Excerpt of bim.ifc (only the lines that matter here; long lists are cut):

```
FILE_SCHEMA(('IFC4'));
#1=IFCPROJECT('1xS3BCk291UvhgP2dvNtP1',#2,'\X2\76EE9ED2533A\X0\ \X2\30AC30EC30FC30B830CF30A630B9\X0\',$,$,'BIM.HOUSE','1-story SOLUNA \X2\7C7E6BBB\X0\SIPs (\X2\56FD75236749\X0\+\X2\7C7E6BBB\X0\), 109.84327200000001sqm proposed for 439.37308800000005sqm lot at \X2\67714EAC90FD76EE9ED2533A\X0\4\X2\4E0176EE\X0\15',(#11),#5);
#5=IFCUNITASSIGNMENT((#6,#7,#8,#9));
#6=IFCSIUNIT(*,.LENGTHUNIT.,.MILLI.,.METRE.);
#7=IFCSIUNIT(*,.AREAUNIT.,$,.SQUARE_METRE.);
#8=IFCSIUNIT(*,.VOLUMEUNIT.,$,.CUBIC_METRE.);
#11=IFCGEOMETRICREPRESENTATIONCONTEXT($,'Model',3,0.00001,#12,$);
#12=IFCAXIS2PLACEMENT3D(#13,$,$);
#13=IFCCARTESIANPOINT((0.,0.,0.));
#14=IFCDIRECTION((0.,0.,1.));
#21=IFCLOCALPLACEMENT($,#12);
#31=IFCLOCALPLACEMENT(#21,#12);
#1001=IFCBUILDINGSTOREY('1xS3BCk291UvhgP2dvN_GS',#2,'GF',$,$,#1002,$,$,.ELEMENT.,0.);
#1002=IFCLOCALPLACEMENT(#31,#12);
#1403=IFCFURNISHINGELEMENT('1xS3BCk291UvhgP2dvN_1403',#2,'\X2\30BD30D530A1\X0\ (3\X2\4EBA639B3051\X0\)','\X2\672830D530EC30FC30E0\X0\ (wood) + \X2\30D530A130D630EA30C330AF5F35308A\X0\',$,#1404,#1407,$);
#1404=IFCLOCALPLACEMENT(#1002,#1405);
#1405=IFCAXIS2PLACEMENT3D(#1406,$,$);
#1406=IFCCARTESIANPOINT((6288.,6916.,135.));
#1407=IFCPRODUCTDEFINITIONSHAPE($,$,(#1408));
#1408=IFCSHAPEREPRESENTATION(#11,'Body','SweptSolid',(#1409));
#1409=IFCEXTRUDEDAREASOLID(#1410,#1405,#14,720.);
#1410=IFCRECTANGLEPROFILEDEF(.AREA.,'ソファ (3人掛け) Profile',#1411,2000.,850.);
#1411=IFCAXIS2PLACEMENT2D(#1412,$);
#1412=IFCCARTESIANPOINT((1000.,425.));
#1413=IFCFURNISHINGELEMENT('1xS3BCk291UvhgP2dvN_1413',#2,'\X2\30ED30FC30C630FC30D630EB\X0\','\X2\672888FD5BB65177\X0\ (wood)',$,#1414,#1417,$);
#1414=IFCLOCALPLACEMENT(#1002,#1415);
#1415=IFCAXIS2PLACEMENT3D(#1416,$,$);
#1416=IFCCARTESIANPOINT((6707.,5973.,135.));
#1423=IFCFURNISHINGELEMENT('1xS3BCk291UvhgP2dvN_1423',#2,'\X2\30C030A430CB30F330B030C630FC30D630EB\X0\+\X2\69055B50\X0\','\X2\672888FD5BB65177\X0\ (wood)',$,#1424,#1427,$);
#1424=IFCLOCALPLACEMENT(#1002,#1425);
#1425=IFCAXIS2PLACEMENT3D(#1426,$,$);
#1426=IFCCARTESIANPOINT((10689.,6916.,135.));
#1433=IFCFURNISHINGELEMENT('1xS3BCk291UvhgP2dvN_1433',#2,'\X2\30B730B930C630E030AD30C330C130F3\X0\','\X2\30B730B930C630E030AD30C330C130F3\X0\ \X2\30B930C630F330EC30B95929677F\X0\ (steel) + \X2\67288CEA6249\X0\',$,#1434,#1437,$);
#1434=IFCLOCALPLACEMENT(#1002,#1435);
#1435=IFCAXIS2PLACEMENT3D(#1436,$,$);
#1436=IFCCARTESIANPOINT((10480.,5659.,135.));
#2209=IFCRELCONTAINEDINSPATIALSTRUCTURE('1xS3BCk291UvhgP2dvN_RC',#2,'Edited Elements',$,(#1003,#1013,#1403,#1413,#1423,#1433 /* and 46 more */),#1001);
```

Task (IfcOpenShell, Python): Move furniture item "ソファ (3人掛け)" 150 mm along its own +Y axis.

```python
import ifcopenshell
import ifcopenshell.api.geometry
import ifcopenshell.util.placement

model = ifcopenshell.open("bim.ifc")

item = model.by_guid("1xS3BCk291UvhgP2dvN_1403")
matrix = ifcopenshell.util.placement.get_local_placement(item.ObjectPlacement)
matrix[:3, 3] += matrix[:3, 1] * 150.0
ifcopenshell.api.geometry.edit_object_placement(model, product=item, matrix=matrix, is_si=False)

print(ifcopenshell.util.placement.get_local_placement(item.ObjectPlacement).round(3) + 0.0)

model.write("bim_rev.ifc")
```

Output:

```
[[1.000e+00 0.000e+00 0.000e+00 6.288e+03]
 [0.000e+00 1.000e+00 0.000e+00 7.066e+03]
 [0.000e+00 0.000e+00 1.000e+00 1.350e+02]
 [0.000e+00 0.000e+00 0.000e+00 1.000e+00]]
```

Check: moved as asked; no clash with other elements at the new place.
